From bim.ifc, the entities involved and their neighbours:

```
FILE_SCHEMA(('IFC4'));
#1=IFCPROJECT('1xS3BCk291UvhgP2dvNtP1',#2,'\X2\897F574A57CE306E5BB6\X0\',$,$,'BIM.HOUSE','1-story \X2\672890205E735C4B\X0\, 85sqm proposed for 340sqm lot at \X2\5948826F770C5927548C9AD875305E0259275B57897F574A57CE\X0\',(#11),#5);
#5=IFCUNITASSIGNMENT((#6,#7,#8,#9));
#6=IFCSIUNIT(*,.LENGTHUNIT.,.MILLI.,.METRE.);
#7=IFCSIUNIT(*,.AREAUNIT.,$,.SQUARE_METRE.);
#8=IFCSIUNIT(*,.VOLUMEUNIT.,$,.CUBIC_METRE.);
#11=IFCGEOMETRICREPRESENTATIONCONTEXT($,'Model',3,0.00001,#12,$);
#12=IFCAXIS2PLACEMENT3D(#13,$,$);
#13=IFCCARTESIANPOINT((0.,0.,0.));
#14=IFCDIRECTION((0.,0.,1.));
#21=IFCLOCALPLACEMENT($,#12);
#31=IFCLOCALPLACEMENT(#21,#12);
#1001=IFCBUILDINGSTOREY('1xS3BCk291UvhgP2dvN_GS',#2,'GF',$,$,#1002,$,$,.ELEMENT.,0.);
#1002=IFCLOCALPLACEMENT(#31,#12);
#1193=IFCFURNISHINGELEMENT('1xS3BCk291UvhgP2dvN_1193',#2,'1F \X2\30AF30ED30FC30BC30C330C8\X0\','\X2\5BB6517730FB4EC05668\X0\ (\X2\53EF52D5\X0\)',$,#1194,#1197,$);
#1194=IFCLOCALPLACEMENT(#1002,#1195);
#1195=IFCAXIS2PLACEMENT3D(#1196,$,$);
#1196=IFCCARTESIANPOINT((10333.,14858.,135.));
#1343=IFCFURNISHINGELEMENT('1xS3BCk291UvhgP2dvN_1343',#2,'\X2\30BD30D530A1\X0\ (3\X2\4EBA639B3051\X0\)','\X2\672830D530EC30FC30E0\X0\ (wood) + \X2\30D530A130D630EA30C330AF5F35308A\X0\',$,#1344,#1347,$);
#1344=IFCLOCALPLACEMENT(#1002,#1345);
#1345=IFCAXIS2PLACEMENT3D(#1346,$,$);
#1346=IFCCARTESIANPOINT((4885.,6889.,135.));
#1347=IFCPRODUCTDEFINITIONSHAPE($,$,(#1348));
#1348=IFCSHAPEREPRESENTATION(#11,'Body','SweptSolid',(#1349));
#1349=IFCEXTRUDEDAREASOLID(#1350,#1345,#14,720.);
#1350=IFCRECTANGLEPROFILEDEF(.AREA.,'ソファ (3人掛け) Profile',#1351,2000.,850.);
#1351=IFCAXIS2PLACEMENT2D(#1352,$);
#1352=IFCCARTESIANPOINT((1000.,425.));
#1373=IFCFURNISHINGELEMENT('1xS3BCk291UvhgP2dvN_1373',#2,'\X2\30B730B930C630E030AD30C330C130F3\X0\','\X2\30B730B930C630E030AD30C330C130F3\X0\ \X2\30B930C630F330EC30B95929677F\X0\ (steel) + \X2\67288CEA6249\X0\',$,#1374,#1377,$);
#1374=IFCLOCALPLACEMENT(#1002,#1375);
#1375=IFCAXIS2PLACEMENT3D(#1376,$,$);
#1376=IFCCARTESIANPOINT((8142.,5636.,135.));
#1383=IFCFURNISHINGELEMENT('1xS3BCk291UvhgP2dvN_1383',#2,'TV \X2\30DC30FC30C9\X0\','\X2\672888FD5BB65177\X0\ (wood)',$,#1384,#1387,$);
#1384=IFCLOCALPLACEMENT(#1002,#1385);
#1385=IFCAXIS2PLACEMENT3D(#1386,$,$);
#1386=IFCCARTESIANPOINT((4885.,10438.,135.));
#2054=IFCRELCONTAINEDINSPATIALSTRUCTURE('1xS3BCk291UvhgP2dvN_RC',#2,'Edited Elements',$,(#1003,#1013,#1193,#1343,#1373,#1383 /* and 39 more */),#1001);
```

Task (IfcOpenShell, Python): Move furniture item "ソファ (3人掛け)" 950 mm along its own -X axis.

```python
import ifcopenshell
import ifcopenshell.api.geometry
import ifcopenshell.util.placement
import ifcopenshell.util.unit

model = ifcopenshell.open("bim.ifc")
unit_scale = ifcopenshell.util.unit.calculate_unit_scale(model)

item = model.by_guid("1xS3BCk291UvhgP2dvN_1343")
matrix = ifcopenshell.util.placement.get_local_placement(item.ObjectPlacement)
matrix[:3, 3] -= matrix[:3, 0] * 0.95 / unit_scale
ifcopenshell.api.geometry.edit_object_placement(model, product=item, matrix=matrix, is_si=False)

print(ifcopenshell.util.placement.get_local_placement(item.ObjectPlacement).round(3) + 0.0)

model.write("bim_v2.ifc")
```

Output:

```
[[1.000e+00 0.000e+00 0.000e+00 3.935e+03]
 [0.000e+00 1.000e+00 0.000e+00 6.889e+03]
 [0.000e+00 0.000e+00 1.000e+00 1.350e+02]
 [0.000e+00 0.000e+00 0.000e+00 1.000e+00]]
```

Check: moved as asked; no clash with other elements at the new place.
